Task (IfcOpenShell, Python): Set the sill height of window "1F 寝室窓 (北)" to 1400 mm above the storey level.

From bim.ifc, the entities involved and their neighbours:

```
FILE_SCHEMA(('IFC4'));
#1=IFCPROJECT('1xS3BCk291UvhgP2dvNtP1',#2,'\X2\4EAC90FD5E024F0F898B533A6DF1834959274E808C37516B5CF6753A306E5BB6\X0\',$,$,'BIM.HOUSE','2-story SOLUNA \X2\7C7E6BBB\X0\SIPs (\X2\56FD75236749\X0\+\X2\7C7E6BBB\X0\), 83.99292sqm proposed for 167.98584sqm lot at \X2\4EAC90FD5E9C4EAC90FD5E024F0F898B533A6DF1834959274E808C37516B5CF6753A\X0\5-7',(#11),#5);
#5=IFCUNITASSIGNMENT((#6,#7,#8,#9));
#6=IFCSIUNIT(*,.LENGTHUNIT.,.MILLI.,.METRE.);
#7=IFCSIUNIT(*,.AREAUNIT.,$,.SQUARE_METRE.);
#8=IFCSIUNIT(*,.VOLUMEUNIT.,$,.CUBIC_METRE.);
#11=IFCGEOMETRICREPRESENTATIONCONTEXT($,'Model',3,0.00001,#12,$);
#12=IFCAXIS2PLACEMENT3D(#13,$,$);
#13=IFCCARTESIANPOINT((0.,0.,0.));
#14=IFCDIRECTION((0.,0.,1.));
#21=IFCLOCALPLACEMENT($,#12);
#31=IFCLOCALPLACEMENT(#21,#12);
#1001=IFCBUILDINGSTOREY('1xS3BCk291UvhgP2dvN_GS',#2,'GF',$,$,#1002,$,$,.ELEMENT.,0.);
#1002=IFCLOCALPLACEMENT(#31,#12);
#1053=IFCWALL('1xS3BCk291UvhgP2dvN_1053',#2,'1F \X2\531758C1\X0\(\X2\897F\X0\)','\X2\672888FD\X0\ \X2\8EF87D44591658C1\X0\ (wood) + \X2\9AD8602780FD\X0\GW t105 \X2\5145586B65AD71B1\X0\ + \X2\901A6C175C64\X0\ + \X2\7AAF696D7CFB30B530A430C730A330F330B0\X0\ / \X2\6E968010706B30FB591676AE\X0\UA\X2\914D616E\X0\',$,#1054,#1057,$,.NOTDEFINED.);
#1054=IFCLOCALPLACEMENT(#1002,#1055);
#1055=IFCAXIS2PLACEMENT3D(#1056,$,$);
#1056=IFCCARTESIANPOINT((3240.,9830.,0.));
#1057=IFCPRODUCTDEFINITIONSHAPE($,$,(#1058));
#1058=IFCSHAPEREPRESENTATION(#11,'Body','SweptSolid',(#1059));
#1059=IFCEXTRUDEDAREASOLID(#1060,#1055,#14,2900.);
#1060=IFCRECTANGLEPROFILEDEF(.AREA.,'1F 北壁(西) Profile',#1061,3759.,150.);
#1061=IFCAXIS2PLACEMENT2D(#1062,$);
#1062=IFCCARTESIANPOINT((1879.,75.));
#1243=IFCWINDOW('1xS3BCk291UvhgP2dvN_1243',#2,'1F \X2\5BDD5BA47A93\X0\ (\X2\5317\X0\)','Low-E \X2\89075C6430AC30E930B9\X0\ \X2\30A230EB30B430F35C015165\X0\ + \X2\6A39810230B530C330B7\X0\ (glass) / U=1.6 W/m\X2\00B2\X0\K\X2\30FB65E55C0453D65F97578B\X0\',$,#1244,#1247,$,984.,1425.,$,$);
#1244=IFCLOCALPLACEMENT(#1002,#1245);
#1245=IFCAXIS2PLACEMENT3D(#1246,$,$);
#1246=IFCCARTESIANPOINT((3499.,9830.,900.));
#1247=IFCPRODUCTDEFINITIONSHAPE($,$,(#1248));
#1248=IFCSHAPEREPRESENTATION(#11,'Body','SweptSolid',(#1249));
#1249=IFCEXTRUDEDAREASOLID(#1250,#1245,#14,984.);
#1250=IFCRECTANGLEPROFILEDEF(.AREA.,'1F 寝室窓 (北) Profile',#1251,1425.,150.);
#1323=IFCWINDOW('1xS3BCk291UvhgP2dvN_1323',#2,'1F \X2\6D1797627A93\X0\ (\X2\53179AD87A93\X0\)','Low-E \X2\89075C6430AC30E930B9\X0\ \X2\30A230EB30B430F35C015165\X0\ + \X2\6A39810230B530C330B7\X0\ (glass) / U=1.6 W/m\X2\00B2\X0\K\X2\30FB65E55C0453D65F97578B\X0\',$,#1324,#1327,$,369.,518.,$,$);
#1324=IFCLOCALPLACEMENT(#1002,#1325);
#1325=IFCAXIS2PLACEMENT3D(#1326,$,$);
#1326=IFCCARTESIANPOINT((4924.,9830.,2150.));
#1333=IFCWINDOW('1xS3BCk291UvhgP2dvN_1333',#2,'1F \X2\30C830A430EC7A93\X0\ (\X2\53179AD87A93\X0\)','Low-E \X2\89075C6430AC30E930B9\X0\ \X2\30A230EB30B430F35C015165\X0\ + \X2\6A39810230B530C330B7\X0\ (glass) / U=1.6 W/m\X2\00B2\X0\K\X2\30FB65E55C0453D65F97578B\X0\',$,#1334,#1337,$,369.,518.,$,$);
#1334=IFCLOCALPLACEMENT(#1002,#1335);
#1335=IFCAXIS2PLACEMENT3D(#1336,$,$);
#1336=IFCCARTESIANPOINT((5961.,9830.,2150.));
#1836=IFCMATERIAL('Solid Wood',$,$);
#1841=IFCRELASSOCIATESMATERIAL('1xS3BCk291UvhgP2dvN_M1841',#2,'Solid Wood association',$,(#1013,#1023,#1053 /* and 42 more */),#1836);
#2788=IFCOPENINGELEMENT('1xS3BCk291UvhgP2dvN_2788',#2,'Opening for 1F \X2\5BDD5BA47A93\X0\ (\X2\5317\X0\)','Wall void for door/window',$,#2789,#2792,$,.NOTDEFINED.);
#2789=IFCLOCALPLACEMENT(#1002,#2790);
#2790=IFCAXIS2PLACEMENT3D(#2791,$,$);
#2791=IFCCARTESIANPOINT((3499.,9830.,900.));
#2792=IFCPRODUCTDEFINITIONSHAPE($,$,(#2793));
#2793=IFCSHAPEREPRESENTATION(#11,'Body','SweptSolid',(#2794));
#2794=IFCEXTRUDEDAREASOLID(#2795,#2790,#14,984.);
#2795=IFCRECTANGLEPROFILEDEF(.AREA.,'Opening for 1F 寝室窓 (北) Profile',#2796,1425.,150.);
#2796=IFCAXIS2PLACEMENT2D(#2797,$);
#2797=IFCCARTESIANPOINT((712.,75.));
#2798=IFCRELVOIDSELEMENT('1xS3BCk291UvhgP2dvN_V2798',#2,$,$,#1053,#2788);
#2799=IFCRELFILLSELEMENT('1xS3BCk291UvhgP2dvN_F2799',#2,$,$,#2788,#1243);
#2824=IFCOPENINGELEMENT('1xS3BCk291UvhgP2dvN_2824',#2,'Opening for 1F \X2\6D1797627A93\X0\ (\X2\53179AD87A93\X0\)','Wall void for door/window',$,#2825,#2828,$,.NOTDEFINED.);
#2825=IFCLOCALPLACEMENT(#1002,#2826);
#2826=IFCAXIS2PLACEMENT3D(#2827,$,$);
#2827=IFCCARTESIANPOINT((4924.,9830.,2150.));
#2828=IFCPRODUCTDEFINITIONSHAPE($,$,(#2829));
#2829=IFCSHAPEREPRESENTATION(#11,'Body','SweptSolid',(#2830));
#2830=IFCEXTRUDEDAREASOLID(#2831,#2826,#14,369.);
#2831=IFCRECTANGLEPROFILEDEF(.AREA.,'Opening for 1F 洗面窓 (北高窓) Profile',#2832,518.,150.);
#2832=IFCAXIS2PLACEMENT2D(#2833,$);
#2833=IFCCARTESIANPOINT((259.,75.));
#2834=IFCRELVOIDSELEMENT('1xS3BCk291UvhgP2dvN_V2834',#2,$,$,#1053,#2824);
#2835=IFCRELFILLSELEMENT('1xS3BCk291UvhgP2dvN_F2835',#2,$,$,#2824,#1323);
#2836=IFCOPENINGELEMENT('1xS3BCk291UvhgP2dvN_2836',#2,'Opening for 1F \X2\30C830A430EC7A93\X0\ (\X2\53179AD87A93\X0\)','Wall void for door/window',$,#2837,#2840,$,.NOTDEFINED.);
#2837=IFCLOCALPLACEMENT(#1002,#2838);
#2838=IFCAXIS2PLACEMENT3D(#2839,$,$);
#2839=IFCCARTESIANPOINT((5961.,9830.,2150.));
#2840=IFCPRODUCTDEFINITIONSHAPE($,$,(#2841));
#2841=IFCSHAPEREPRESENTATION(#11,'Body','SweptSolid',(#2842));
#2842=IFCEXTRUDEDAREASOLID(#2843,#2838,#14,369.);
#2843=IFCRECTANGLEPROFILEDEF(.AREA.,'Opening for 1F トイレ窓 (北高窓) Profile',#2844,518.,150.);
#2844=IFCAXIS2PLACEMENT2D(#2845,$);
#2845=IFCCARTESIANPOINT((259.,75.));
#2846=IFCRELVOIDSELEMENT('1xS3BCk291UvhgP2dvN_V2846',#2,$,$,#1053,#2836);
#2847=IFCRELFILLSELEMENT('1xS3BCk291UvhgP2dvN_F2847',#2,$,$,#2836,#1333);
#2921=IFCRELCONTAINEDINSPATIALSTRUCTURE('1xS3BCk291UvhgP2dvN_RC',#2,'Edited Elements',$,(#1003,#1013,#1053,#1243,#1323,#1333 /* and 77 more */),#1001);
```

```python
import numpy as np
import ifcopenshell
import ifcopenshell.api.geometry
import ifcopenshell.geom
import ifcopenshell.util.element
import ifcopenshell.util.placement
import ifcopenshell.util.shape
import ifcopenshell.util.unit

model = ifcopenshell.open("bim.ifc")
unit_scale = ifcopenshell.util.unit.calculate_unit_scale(model)

window = model.by_guid("1xS3BCk291UvhgP2dvN_1243")
opening = window.FillsVoids[0].RelatingOpeningElement
storey = ifcopenshell.util.element.get_container(window, ifc_class="IfcBuildingStorey")
level = ifcopenshell.util.placement.get_local_placement(storey.ObjectPlacement)[2, 3]

# The opening's origin need not be at the sill, so measure its lowest point.
shape = ifcopenshell.geom.create_shape(ifcopenshell.geom.settings(), opening)
bottom = ifcopenshell.util.shape.get_shape_bottom_elevation(shape, shape.geometry) / unit_scale
dz = level + 1.4 / unit_scale - bottom

shift = np.array([0.0, 0.0, dz])
# The window is not placed relative to its opening, so move both.
for product in (opening, window):
    matrix = ifcopenshell.util.placement.get_local_placement(product.ObjectPlacement)
    matrix[:3, 3] += shift
    ifcopenshell.api.geometry.edit_object_placement(model, product=product, matrix=matrix, is_si=False)

print(f"moved by {dz * unit_scale:+.3f} m")

model.write("bim_updated.ifc")
```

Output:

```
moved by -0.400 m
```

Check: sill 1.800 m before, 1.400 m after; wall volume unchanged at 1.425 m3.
